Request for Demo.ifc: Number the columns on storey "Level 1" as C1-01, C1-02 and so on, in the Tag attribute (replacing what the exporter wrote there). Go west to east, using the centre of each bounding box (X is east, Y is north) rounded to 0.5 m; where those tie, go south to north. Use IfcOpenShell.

First a look at what the model holds.

```python
import ifcopenshell
import ifcopenshell.util.element
import ifcopenshell.util.placement

model = ifcopenshell.open("Demo.ifc")
print(model.schema)
storey = next(s for s in model.by_type("IfcBuildingStorey") if s.Name == "Level 1")
columns = [e for e in ifcopenshell.util.element.get_decomposition(storey) if e.is_a("IfcColumn")]
for e in sorted(columns, key=lambda e: e.id()):
    origin = ifcopenshell.util.placement.get_local_placement(e.ObjectPlacement)[:3, 3]
    print(e.id(), e.Tag, e.Name, origin.round(2) + 0.0, sep=" | ")
```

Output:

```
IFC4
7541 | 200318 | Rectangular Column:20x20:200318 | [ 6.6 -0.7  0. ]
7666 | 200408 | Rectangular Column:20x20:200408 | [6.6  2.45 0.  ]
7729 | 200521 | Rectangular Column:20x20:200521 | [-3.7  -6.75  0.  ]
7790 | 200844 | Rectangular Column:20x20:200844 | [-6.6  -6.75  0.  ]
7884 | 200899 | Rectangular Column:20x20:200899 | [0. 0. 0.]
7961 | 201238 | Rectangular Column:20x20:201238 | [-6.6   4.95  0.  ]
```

```python
import ifcopenshell
import ifcopenshell.geom
import ifcopenshell.util.element
import ifcopenshell.util.shape

model = ifcopenshell.open("Demo.ifc")
settings = ifcopenshell.geom.settings()
settings.set("use-world-coords", True)


def centre(element):
    shape = ifcopenshell.geom.create_shape(settings, element)
    return ifcopenshell.util.shape.get_bbox_centroid(shape.geometry)


storey = next(s for s in model.by_type("IfcBuildingStorey") if s.Name == "Level 1")
columns = [e for e in ifcopenshell.util.element.get_decomposition(storey) if e.is_a("IfcColumn")]

# Insertion points can sit at a corner or the storey origin, so sort by the geometry (in metres).
centres = {e: centre(e) for e in columns}
columns.sort(key=lambda e: (round(centres[e][0] / 0.5), centres[e][1]))

for i, e in enumerate(columns, start=1):
    number = f"C1-{i:02d}"
    e.Tag = number
    print(e.id(), number)

model.write("Demo_updated.ifc")
```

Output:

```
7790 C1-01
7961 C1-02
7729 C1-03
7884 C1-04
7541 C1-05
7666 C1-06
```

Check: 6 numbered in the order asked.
